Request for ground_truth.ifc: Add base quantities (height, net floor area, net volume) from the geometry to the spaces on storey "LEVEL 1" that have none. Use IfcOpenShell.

First a look at what the model holds.

```python
import ifcopenshell
import ifcopenshell.util.element
import ifcopenshell.util.unit

model = ifcopenshell.open("ground_truth.ifc")
print(model.schema)
for unit_type in ("LENGTHUNIT", "AREAUNIT", "VOLUMEUNIT"):
    print(unit_type, ifcopenshell.util.unit.calculate_unit_scale(model, unit_type))
storey = next(s for s in model.by_type("IfcBuildingStorey") if s.Name == "LEVEL 1")
spaces = [e for e in ifcopenshell.util.element.get_decomposition(storey) if e.is_a("IfcSpace")]
for e in sorted(spaces, key=lambda e: e.id()):
    print(e.id(), e.is_a(), e.Name, list(ifcopenshell.util.element.get_psets(e, qtos_only=True)), sep=" | ")
```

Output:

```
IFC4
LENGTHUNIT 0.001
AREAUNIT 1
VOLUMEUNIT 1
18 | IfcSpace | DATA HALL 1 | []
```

```python
import ifcopenshell
import ifcopenshell.api.pset
import ifcopenshell.geom
import ifcopenshell.util.element
import ifcopenshell.util.shape
import ifcopenshell.util.unit

model = ifcopenshell.open("ground_truth.ifc")
unit_scale = ifcopenshell.util.unit.calculate_unit_scale(model)
area_scale = ifcopenshell.util.unit.calculate_unit_scale(model, "AREAUNIT")
volume_scale = ifcopenshell.util.unit.calculate_unit_scale(model, "VOLUMEUNIT")
settings = ifcopenshell.geom.settings()

storey = next(s for s in model.by_type("IfcBuildingStorey") if s.Name == "LEVEL 1")
spaces = [e for e in ifcopenshell.util.element.get_decomposition(storey) if e.is_a("IfcSpace")]

for e in sorted(spaces, key=lambda e: e.id()):
    if ifcopenshell.util.element.get_psets(e, qtos_only=True, should_inherit=False):
        continue
    # Geometry comes back in metres, in the element's own axes.
    shape = ifcopenshell.geom.create_shape(settings, e)
    values = {
        "Height": ifcopenshell.util.shape.get_z(shape.geometry) / unit_scale,
        "NetFloorArea": ifcopenshell.util.shape.get_footprint_area(shape.geometry) / area_scale,
        "NetVolume": ifcopenshell.util.shape.get_volume(shape.geometry) / volume_scale,
    }
    qto = ifcopenshell.api.pset.add_qto(model, product=e, name="Qto_SpaceBaseQuantities")
    ifcopenshell.api.pset.edit_qto(model, qto=qto, properties=values)
    print(e.id(), {k: round(v, 3) for k, v in values.items()})

model.write("ground_truth-out.ifc")
```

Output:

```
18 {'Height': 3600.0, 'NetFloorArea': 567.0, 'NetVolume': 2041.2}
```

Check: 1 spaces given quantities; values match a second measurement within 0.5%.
